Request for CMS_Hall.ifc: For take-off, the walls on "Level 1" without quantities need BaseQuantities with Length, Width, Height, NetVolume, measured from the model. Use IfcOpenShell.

First a look at what the model holds.

```python
import ifcopenshell
import ifcopenshell.util.element
import ifcopenshell.util.unit

model = ifcopenshell.open("CMS_Hall.ifc")
print(model.schema)
for unit_type in ("LENGTHUNIT", "AREAUNIT", "VOLUMEUNIT"):
    print(unit_type, ifcopenshell.util.unit.calculate_unit_scale(model, unit_type))
storey = next(s for s in model.by_type("IfcBuildingStorey") if s.Name == "Level 1")
walls = [e for e in ifcopenshell.util.element.get_decomposition(storey) if e.is_a("IfcWall")]
for e in sorted(walls, key=lambda e: e.id()):
    print(e.id(), e.is_a(), e.Name, list(ifcopenshell.util.element.get_psets(e, qtos_only=True)), sep=" | ")
```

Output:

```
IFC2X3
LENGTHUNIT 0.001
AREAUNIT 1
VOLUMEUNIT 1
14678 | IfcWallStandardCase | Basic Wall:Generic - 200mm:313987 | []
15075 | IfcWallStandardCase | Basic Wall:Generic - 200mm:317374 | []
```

```python
import ifcopenshell
import ifcopenshell.api.pset
import ifcopenshell.geom
import ifcopenshell.util.element
import ifcopenshell.util.shape
import ifcopenshell.util.unit

model = ifcopenshell.open("CMS_Hall.ifc")
unit_scale = ifcopenshell.util.unit.calculate_unit_scale(model)
volume_scale = ifcopenshell.util.unit.calculate_unit_scale(model, "VOLUMEUNIT")
settings = ifcopenshell.geom.settings()

storey = next(s for s in model.by_type("IfcBuildingStorey") if s.Name == "Level 1")
walls = [e for e in ifcopenshell.util.element.get_decomposition(storey) if e.is_a("IfcWall")]

for e in sorted(walls, key=lambda e: e.id()):
    if ifcopenshell.util.element.get_psets(e, qtos_only=True, should_inherit=False):
        continue
    # Geometry comes back in metres, in the element's own axes.
    shape = ifcopenshell.geom.create_shape(settings, e)
    values = {
        "Length": ifcopenshell.util.shape.get_x(shape.geometry) / unit_scale,
        "Width": ifcopenshell.util.shape.get_y(shape.geometry) / unit_scale,
        "Height": ifcopenshell.util.shape.get_z(shape.geometry) / unit_scale,
        "NetVolume": ifcopenshell.util.shape.get_volume(shape.geometry) / volume_scale,
    }
    qto = ifcopenshell.api.pset.add_qto(model, product=e, name="BaseQuantities")
    ifcopenshell.api.pset.edit_qto(model, qto=qto, properties=values)
    print(e.id(), {k: round(v, 3) for k, v in values.items()})

model.write("CMS_Hall_rev.ifc")
```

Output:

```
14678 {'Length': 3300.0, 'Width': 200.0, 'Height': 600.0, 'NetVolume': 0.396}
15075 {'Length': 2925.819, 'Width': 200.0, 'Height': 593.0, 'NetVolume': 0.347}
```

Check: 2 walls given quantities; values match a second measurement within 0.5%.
